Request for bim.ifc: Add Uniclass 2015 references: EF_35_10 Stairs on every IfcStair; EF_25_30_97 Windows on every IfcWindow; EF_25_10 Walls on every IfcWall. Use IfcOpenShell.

First a look at what the model holds.

```python
import ifcopenshell

model = ifcopenshell.open("bim.ifc")
print(model.schema)
print("classifications:", [c.Name for c in model.by_type("IfcClassification")])
for ifc_class in ("IfcDoor", "IfcRoof", "IfcStair", "IfcWall", "IfcWindow"):
    print(ifc_class, len(model.by_type(ifc_class)))
```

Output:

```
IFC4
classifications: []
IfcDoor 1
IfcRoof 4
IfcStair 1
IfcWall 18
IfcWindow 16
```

```python
import ifcopenshell
import ifcopenshell.api.classification

model = ifcopenshell.open("bim.ifc")

system = ifcopenshell.api.classification.add_classification(model, classification="Uniclass 2015")

codes = {
    "IfcStair": ("EF_35_10", "Stairs"),
    "IfcWindow": ("EF_25_30_97", "Windows"),
    "IfcWall": ("EF_25_10", "Walls"),
}
for ifc_class, (code, name) in codes.items():
    products = model.by_type(ifc_class)
    ifcopenshell.api.classification.add_reference(
        model, products=products, classification=system, identification=code, name=name
    )
    print(code, len(products))

model.write("bim_edited.ifc")
```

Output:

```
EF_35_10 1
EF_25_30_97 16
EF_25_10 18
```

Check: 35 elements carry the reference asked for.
